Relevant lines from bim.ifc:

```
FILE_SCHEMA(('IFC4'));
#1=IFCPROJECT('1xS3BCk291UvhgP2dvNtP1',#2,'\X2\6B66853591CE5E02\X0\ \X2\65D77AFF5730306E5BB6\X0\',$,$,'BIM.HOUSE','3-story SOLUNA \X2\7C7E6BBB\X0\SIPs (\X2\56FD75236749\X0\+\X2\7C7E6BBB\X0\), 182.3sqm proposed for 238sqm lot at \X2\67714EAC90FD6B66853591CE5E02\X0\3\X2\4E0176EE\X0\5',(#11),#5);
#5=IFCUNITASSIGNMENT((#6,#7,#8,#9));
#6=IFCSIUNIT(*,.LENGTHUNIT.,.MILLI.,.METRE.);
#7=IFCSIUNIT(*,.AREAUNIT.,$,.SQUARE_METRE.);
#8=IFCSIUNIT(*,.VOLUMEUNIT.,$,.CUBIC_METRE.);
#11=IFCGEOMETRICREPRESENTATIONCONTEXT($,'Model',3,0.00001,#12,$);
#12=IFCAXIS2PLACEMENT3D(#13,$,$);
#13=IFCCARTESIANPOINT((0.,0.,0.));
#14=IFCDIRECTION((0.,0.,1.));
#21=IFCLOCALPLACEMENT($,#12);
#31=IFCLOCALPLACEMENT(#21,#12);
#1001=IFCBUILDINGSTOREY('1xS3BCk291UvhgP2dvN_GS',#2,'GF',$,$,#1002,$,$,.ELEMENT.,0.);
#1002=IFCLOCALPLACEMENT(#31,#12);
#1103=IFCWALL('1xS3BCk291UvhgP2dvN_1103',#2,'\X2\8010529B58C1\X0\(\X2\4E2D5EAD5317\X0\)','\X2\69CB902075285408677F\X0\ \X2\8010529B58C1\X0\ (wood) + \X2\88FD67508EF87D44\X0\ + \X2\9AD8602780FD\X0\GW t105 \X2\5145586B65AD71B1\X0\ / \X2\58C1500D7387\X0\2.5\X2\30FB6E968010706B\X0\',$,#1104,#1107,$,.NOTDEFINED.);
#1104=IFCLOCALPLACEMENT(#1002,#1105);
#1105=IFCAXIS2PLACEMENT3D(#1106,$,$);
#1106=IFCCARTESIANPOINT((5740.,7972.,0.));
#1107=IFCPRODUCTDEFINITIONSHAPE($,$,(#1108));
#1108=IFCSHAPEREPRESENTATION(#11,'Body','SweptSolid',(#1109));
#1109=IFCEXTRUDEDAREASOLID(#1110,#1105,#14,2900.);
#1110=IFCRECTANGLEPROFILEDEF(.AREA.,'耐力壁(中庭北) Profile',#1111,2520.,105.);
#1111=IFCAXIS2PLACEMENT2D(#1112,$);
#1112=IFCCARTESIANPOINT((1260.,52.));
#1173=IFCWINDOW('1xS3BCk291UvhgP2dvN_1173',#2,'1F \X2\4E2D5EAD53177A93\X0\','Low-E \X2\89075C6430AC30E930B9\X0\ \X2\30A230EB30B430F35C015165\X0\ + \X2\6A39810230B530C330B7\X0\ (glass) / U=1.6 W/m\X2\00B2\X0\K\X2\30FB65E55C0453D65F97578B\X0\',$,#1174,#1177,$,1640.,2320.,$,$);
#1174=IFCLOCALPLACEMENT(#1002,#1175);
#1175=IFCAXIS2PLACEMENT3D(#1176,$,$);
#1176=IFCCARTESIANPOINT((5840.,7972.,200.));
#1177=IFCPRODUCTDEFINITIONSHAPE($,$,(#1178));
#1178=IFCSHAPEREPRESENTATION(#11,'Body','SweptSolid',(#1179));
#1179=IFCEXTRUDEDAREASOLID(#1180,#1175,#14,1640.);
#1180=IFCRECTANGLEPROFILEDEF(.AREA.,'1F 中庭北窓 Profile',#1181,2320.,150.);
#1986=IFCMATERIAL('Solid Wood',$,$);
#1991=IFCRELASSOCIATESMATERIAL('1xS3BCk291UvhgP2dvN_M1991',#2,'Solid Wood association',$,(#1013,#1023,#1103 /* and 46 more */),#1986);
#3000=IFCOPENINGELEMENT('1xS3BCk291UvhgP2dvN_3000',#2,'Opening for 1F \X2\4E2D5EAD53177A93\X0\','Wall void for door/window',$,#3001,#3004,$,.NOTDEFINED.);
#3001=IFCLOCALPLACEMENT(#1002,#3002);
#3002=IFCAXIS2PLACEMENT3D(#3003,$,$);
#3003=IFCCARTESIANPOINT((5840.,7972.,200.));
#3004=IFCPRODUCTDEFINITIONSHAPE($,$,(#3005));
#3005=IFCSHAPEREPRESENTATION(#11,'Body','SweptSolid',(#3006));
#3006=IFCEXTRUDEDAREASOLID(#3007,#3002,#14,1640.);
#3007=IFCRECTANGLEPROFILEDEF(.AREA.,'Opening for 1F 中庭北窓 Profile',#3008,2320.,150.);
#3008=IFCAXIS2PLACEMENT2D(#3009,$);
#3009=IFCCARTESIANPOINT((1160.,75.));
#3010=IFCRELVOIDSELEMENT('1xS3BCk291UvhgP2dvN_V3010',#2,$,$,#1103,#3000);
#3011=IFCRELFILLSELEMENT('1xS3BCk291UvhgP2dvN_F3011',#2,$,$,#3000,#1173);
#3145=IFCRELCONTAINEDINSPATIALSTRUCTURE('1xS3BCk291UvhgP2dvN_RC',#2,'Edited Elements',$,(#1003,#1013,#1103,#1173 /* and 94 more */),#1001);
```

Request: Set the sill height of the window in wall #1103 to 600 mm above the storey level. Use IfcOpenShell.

```python
import numpy as np
import ifcopenshell
import ifcopenshell.api.geometry
import ifcopenshell.geom
import ifcopenshell.util.element
import ifcopenshell.util.placement
import ifcopenshell.util.shape
import ifcopenshell.util.unit

model = ifcopenshell.open("bim.ifc")
unit_scale = ifcopenshell.util.unit.calculate_unit_scale(model)

window = model.by_guid("1xS3BCk291UvhgP2dvN_1173")
opening = window.FillsVoids[0].RelatingOpeningElement
storey = ifcopenshell.util.element.get_container(window, ifc_class="IfcBuildingStorey")
level = ifcopenshell.util.placement.get_local_placement(storey.ObjectPlacement)[2, 3]

# The opening's origin need not be at the sill, so measure its lowest point.
shape = ifcopenshell.geom.create_shape(ifcopenshell.geom.settings(), opening)
bottom = ifcopenshell.util.shape.get_shape_bottom_elevation(shape, shape.geometry) / unit_scale
dz = level + 0.6 / unit_scale - bottom

shift = np.array([0.0, 0.0, dz])
# The window is not placed relative to its opening, so move both.
for product in (opening, window):
    matrix = ifcopenshell.util.placement.get_local_placement(product.ObjectPlacement)
    matrix[:3, 3] += shift
    ifcopenshell.api.geometry.edit_object_placement(model, product=product, matrix=matrix, is_si=False)

print(f"moved by {dz * unit_scale:+.3f} m")

model.write("bim_updated.ifc")
```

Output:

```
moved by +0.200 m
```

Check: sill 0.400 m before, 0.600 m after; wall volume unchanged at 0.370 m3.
